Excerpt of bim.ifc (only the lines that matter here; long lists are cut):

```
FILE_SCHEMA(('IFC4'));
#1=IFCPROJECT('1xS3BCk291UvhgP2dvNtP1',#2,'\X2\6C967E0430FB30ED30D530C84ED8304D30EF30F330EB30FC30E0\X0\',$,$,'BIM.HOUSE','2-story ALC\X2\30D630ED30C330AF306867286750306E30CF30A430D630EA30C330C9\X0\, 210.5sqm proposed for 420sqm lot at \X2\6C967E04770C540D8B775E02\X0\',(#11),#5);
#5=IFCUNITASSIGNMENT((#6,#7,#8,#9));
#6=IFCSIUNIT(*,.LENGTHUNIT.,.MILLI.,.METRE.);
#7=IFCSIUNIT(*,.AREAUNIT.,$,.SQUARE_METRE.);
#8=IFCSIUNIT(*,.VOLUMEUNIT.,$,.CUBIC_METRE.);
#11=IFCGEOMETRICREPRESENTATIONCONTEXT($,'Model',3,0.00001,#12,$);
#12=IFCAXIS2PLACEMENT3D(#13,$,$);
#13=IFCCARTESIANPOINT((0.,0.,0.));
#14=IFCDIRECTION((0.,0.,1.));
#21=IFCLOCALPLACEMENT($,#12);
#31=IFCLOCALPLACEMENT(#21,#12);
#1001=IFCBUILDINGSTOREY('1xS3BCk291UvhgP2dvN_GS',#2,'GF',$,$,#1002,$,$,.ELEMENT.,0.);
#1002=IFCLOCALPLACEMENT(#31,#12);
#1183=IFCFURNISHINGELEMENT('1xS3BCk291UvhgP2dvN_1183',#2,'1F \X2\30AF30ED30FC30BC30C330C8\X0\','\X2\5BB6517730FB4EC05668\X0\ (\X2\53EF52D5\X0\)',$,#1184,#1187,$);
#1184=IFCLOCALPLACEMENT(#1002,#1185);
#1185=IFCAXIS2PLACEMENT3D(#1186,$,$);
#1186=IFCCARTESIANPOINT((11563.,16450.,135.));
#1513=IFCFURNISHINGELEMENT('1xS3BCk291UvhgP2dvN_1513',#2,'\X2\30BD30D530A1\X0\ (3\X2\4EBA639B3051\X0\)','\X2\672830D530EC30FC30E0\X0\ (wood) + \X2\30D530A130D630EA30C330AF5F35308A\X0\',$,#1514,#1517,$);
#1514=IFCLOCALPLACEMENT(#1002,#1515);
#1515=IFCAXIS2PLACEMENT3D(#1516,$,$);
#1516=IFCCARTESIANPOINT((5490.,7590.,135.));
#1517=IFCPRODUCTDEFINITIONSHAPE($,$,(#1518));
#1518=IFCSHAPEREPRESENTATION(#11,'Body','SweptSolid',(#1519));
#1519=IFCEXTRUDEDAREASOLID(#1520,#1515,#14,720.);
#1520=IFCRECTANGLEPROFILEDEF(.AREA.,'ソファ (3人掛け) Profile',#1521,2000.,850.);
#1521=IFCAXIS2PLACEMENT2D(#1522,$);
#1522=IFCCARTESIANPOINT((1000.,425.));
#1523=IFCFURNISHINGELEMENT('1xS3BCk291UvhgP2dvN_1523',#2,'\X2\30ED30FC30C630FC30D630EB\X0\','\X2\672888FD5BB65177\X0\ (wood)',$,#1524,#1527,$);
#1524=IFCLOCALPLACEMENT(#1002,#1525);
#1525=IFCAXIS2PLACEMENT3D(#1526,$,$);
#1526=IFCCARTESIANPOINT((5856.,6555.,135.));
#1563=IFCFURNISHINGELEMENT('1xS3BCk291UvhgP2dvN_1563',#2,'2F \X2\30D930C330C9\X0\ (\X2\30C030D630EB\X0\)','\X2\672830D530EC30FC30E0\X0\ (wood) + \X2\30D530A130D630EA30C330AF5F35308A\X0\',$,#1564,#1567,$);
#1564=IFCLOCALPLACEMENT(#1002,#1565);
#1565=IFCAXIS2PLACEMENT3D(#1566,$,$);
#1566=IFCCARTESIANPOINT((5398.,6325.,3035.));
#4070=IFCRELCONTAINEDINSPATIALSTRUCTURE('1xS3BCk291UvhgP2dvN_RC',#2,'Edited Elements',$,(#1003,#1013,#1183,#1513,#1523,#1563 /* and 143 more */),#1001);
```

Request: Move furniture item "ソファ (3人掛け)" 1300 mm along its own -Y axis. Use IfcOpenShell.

```python
import ifcopenshell
import ifcopenshell.api.geometry
import ifcopenshell.util.placement
import ifcopenshell.util.unit

model = ifcopenshell.open("bim.ifc")
unit_scale = ifcopenshell.util.unit.calculate_unit_scale(model)

item = model.by_guid("1xS3BCk291UvhgP2dvN_1513")
matrix = ifcopenshell.util.placement.get_local_placement(item.ObjectPlacement)
matrix[:3, 3] -= matrix[:3, 1] * 1.3 / unit_scale
ifcopenshell.api.geometry.edit_object_placement(model, product=item, matrix=matrix, is_si=False)

print(ifcopenshell.util.placement.get_local_placement(item.ObjectPlacement).round(3) + 0.0)

model.write("bim_v2.ifc")
```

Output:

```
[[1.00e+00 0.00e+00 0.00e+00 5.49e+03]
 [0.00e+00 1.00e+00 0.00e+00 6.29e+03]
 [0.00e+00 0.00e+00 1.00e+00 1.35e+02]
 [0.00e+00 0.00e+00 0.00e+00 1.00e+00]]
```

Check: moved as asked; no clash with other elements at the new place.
